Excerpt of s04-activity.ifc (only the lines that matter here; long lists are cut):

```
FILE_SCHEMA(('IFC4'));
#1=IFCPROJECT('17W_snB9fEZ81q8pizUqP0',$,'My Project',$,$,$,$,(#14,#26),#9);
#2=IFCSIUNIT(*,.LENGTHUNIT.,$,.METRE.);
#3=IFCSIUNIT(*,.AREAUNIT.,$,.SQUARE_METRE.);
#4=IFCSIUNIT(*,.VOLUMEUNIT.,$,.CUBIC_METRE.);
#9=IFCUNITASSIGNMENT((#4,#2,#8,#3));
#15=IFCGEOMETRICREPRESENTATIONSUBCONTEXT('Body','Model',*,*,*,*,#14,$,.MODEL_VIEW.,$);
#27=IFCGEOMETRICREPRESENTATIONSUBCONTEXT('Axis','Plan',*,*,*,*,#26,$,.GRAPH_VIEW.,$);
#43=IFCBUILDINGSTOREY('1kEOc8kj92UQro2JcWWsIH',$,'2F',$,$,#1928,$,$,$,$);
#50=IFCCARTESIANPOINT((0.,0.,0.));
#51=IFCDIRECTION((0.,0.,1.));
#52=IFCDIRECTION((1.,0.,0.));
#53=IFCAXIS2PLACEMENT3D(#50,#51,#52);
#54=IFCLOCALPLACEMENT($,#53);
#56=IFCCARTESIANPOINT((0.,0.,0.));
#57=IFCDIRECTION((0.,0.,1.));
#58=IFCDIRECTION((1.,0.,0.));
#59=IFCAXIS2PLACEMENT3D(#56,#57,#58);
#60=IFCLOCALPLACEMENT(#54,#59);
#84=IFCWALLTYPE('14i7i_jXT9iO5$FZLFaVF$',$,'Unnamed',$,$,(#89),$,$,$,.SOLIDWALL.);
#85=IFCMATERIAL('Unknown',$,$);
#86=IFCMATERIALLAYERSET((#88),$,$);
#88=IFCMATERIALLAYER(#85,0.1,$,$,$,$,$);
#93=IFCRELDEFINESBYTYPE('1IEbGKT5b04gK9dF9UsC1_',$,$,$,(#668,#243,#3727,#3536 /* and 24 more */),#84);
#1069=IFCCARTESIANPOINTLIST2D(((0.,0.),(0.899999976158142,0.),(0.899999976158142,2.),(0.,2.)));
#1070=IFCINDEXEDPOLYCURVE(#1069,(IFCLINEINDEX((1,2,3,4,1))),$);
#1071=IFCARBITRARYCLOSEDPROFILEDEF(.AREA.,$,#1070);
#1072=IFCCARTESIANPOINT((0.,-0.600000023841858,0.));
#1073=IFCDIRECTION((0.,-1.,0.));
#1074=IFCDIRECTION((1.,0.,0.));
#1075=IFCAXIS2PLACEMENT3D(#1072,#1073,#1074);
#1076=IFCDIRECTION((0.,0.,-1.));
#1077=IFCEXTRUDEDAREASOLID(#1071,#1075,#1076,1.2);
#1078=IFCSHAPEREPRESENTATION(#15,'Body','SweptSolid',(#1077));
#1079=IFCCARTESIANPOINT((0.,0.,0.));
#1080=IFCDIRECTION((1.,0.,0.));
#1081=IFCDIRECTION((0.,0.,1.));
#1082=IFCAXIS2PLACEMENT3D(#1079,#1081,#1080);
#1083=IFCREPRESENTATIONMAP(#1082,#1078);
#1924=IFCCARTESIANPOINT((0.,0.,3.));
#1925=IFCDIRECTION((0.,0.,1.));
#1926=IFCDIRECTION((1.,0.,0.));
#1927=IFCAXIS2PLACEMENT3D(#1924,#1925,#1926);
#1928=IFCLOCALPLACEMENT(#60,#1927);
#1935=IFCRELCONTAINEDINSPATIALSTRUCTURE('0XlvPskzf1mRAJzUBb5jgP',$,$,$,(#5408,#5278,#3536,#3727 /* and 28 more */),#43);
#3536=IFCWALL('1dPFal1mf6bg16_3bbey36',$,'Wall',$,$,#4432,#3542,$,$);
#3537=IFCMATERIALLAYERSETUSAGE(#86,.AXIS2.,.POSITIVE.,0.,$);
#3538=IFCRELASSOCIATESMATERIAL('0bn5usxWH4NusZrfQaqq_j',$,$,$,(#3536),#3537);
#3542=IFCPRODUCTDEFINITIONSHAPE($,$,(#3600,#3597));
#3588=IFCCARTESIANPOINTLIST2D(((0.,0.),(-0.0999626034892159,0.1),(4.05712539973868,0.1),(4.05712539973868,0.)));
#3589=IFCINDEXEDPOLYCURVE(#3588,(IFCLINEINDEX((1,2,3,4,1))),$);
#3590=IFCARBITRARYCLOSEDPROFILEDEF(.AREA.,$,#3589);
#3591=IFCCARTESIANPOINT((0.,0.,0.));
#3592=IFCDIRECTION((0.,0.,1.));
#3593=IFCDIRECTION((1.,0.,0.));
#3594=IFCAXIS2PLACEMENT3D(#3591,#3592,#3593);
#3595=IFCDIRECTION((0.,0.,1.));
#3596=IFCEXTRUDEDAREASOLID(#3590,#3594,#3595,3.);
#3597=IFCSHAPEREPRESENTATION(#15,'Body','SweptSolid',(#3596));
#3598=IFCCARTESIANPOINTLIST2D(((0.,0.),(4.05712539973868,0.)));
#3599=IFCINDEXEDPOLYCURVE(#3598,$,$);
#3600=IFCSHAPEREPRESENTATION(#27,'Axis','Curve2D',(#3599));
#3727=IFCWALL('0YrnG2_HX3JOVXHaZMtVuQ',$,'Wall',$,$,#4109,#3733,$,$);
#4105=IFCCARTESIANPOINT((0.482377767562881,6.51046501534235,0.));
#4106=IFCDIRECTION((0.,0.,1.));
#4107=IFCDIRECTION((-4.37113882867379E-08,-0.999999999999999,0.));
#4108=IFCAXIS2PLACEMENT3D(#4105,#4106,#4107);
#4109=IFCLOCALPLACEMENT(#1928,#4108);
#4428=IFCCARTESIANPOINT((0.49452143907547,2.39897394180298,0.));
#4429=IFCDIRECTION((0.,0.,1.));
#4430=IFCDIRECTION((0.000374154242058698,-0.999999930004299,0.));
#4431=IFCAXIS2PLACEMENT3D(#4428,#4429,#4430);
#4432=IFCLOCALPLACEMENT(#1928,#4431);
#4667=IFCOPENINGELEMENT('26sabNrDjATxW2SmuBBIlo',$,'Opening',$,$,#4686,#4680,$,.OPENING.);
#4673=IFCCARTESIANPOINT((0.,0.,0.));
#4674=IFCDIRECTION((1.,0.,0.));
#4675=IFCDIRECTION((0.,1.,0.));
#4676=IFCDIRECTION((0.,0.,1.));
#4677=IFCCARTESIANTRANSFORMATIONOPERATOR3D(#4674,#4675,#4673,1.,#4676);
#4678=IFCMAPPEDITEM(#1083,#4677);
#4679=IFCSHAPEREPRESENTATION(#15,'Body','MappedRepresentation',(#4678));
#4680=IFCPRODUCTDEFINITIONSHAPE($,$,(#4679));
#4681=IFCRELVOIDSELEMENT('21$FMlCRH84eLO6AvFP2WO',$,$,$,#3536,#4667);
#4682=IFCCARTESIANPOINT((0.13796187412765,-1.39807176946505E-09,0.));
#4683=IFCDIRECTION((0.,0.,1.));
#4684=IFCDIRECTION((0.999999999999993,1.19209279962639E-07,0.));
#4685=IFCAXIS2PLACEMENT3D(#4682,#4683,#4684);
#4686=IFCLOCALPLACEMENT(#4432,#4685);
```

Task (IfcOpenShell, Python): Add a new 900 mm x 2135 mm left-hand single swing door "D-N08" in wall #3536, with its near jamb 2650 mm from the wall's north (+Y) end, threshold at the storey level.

```python
import numpy as np
import ifcopenshell
import ifcopenshell.api.feature
import ifcopenshell.api.geometry
import ifcopenshell.api.root
import ifcopenshell.api.spatial
import ifcopenshell.geom
import ifcopenshell.util.element
import ifcopenshell.util.placement
import ifcopenshell.util.representation
import ifcopenshell.util.shape
import ifcopenshell.util.unit

model = ifcopenshell.open("s04-activity.ifc")
unit_scale = ifcopenshell.util.unit.calculate_unit_scale(model)
settings = ifcopenshell.geom.settings()


def volume(element):
    """Net volume in cubic metres, openings subtracted."""
    shape = ifcopenshell.geom.create_shape(settings, element)
    return ifcopenshell.util.shape.get_volume(shape.geometry)


wall = model.by_guid("1dPFal1mf6bg16_3bbey36")
storey = ifcopenshell.util.element.get_container(wall, ifc_class="IfcBuildingStorey")
context = ifcopenshell.util.representation.get_context(model, "Model", "Body", "MODEL_VIEW")
before = volume(wall)

width, height, from_end, sill = 0.9, 2.135, 2.65, 0.0  # metres

# The wall runs along its own X axis, and the end named is its -X end.
wall_shape = ifcopenshell.geom.create_shape(settings, wall)
x, y, z = ifcopenshell.util.shape.get_vertices(wall_shape.geometry).T
start = x.min() + from_end
face, thickness = float(y.min()), float(y.max() - y.min())
wall_matrix = ifcopenshell.util.placement.get_local_placement(wall.ObjectPlacement)
level = ifcopenshell.util.placement.get_local_placement(storey.ObjectPlacement)[2, 3]


def in_wall(x, y):
    """Placement at x, y metres in the wall's axes, at sill height."""
    matrix = wall_matrix.copy()
    matrix[:, 3] = wall_matrix @ np.array([x / unit_scale, y / unit_scale, 0.0, 1.0])
    matrix[2, 3] = level + sill / unit_scale
    return matrix


# Opening: a box that overshoots both wall faces by 50 mm.
opening = ifcopenshell.api.root.create_entity(model, ifc_class="IfcOpeningElement", predefined_type="OPENING")
box = ifcopenshell.api.geometry.add_wall_representation(
    model, context=context, length=width, height=height, thickness=thickness + 0.1
)
ifcopenshell.api.geometry.assign_representation(model, product=opening, representation=box)
ifcopenshell.api.geometry.edit_object_placement(model, product=opening, matrix=in_wall(start, face - 0.05), is_si=False)
ifcopenshell.api.feature.add_feature(model, feature=opening, element=wall)

door = ifcopenshell.api.root.create_entity(model, ifc_class="IfcDoor", name="D-N08", predefined_type="DOOR")
door.OverallWidth, door.OverallHeight = width / unit_scale, height / unit_scale
door.OperationType = "SINGLE_SWING_LEFT"
body = ifcopenshell.api.geometry.add_door_representation(
    model,
    context=context,
    overall_width=door.OverallWidth,
    overall_height=door.OverallHeight,
    operation_type="SINGLE_SWING_LEFT",
    lining_properties={"LiningDepth": thickness / unit_scale, "ThresholdDepth": thickness / unit_scale},
)
ifcopenshell.api.geometry.assign_representation(model, product=door, representation=body)
ifcopenshell.api.spatial.assign_container(model, products=[door], relating_structure=storey)
ifcopenshell.api.feature.add_filling(model, opening=opening, element=door)

# The lining spans the wall, so the door starts at the wall face.
ifcopenshell.api.geometry.edit_object_placement(model, product=door, matrix=in_wall(start, face), is_si=False)

after = volume(wall)

print(f"wall volume {before:.3f} -> {after:.3f} m3")

model.write("s04-activity-out.ifc")
```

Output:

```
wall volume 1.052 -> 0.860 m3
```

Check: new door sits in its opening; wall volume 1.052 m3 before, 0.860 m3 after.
